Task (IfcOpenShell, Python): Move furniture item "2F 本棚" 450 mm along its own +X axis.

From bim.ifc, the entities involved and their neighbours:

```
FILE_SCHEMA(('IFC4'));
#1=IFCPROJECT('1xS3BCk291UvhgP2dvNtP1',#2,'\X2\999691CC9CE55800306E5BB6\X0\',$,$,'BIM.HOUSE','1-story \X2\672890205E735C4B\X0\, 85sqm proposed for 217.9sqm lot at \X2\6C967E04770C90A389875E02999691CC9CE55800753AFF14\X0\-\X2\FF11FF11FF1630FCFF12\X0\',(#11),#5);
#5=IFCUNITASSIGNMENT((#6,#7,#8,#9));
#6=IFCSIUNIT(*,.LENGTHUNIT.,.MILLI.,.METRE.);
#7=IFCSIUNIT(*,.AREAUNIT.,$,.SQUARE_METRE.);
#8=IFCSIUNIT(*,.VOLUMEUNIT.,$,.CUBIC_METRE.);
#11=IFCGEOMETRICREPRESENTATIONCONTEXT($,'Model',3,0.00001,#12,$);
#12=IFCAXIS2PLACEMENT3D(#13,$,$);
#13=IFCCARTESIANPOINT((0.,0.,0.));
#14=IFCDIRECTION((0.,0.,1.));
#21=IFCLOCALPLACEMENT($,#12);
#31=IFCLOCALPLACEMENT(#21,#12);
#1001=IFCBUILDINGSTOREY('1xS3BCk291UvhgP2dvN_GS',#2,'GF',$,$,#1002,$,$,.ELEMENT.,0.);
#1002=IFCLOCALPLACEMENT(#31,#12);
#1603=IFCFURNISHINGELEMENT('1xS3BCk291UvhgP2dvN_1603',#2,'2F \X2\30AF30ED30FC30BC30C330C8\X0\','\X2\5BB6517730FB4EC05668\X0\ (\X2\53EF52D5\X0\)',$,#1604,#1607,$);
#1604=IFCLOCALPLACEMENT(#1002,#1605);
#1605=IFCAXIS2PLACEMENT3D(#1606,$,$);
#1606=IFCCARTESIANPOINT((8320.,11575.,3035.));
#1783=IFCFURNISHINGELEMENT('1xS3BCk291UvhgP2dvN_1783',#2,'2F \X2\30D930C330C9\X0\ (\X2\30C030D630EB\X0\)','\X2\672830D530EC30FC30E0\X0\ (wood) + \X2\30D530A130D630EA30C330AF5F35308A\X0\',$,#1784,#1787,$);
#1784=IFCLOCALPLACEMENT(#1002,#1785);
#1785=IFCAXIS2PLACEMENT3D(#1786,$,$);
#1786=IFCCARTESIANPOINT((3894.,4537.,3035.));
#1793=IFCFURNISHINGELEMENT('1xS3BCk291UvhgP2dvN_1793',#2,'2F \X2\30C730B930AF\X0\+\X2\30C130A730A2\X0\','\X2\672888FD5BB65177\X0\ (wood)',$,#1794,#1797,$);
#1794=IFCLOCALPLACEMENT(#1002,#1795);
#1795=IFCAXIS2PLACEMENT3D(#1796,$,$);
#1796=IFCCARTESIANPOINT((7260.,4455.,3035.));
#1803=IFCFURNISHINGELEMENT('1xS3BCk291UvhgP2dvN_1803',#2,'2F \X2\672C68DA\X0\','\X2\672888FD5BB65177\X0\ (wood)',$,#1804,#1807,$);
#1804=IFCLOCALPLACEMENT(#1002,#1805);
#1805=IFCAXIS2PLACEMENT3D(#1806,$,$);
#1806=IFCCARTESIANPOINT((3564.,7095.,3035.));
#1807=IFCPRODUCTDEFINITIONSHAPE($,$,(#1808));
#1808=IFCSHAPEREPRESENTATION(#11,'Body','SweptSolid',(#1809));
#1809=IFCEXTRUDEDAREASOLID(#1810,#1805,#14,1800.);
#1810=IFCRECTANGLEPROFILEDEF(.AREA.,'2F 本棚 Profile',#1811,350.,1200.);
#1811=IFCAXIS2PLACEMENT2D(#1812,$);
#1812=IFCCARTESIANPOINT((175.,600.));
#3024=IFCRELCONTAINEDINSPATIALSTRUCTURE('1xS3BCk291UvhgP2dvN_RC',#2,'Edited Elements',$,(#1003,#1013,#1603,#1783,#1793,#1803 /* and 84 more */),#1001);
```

```python
import ifcopenshell
import ifcopenshell.api.geometry
import ifcopenshell.util.placement

model = ifcopenshell.open("bim.ifc")

item = model.by_guid("1xS3BCk291UvhgP2dvN_1803")
matrix = ifcopenshell.util.placement.get_local_placement(item.ObjectPlacement)
matrix[:3, 3] += matrix[:3, 0] * 450.0
ifcopenshell.api.geometry.edit_object_placement(model, product=item, matrix=matrix, is_si=False)

print(ifcopenshell.util.placement.get_local_placement(item.ObjectPlacement).round(3) + 0.0)

model.write("bim_updated.ifc")
```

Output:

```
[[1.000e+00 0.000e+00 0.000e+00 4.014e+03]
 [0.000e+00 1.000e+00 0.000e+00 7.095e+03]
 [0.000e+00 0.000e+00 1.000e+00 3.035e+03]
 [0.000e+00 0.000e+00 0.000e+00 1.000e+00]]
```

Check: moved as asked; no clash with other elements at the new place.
